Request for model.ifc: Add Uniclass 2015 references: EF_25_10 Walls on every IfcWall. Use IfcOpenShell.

First a look at what the model holds.

```python
import ifcopenshell

model = ifcopenshell.open("model.ifc")
print(model.schema)
print("classifications:", [c.Name for c in model.by_type("IfcClassification")])
for ifc_class in ("IfcDoor", "IfcRoof", "IfcStair", "IfcWall", "IfcWindow"):
    print(ifc_class, len(model.by_type(ifc_class)))
```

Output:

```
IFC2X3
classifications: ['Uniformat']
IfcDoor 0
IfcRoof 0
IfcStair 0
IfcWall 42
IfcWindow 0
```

```python
import ifcopenshell
import ifcopenshell.api.classification

model = ifcopenshell.open("model.ifc")

# IFC2X3 requires Source and Edition and has no link from the project to the system.
system = model.create_entity("IfcClassification", Source="NBS", Edition="2015", Name="Uniclass 2015")

codes = {
    "IfcWall": ("EF_25_10", "Walls"),
}
for ifc_class, (code, name) in codes.items():
    products = model.by_type(ifc_class)
    ifcopenshell.api.classification.add_reference(
        model, products=products, classification=system, identification=code, name=name
    )
    print(code, len(products))

model.write("model_edited.ifc")
```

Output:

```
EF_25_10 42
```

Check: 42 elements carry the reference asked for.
